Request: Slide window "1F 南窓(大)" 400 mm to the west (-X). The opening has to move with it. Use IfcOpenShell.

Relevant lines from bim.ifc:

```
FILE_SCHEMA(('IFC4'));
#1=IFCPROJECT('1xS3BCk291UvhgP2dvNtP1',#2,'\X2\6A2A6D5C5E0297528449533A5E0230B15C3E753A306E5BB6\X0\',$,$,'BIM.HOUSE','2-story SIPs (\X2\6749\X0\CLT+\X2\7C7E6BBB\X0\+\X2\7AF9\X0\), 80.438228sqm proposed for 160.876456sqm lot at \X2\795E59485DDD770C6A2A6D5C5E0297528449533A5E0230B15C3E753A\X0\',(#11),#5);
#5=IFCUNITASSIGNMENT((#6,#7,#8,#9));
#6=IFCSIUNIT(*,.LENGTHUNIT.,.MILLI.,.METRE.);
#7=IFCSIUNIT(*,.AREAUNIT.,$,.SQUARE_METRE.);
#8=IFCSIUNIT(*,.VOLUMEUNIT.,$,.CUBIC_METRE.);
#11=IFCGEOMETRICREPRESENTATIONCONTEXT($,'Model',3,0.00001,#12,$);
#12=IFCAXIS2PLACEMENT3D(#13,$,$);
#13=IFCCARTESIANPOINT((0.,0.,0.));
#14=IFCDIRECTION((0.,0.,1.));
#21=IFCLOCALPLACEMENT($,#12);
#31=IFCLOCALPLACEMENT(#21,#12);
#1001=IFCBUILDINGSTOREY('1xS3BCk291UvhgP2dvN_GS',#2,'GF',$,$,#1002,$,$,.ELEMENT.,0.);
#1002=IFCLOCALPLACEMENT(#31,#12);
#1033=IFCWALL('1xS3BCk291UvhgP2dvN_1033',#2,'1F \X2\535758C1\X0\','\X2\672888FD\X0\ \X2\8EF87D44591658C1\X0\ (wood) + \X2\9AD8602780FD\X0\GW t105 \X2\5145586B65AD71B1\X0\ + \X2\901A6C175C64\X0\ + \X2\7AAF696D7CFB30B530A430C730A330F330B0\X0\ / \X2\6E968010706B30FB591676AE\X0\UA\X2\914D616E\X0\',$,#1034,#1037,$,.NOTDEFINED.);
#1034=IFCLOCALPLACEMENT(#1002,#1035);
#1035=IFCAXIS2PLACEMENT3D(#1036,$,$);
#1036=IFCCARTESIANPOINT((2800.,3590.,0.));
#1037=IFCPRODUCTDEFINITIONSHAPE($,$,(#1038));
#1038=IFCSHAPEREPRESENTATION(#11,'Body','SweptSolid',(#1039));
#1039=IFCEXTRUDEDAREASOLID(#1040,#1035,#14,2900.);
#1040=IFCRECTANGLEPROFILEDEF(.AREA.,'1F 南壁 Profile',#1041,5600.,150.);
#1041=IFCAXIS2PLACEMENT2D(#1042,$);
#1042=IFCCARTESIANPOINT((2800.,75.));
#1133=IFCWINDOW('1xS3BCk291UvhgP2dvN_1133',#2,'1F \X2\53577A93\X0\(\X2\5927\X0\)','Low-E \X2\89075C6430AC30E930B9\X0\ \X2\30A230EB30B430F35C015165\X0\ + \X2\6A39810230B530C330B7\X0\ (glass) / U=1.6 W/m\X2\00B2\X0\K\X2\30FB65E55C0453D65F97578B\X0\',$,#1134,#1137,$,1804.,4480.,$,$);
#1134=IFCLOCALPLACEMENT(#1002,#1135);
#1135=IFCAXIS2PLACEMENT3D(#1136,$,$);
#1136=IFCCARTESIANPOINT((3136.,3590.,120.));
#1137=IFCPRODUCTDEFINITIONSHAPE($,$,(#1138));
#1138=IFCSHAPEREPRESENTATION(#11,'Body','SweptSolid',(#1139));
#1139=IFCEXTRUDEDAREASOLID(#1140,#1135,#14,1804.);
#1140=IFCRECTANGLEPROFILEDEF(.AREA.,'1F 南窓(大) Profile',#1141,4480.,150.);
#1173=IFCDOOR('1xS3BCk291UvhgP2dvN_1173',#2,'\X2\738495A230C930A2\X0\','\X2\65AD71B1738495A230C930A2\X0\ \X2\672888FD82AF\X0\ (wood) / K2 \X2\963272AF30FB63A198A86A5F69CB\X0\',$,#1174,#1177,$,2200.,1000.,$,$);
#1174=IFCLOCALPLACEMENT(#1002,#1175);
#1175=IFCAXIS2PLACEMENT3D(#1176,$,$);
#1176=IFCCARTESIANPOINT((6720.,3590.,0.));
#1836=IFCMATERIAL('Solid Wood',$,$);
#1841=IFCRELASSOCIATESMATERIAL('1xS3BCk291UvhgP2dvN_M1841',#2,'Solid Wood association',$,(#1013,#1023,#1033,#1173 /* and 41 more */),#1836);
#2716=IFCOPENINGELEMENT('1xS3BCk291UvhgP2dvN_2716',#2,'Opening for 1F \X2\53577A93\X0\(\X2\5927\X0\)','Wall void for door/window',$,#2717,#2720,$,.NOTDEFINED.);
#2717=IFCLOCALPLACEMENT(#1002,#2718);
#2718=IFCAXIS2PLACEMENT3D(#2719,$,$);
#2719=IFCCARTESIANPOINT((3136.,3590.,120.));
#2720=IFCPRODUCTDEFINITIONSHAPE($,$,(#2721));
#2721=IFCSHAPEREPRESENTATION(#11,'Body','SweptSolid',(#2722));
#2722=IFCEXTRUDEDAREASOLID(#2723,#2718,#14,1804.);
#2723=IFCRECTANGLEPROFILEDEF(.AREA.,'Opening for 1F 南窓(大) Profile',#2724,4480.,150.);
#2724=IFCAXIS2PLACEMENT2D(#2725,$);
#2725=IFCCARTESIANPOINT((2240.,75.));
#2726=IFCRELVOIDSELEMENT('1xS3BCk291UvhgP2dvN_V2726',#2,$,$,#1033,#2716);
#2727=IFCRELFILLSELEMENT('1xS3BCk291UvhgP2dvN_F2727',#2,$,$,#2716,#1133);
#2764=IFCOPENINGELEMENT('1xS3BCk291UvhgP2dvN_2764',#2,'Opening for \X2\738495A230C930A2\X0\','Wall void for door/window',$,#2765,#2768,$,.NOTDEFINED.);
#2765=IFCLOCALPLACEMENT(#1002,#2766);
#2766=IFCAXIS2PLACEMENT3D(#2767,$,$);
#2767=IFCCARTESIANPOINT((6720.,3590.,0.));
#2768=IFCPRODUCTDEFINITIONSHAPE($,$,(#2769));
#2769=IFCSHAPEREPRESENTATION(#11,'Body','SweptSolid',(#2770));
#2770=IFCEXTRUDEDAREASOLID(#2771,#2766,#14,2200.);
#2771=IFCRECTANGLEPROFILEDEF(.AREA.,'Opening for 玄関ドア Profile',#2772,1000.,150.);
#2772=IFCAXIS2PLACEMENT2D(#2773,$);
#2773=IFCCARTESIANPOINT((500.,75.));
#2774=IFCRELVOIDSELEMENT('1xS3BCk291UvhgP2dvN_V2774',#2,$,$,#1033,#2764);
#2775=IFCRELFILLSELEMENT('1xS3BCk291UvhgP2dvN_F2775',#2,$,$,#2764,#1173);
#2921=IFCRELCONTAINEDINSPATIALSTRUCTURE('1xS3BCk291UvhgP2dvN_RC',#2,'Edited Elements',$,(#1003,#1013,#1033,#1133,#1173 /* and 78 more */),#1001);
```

```python
import ifcopenshell
import ifcopenshell.api.geometry
import ifcopenshell.util.placement
import ifcopenshell.util.unit

model = ifcopenshell.open("bim.ifc")
unit_scale = ifcopenshell.util.unit.calculate_unit_scale(model)

window = model.by_id(1133)
opening = window.FillsVoids[0].RelatingOpeningElement
wall = opening.VoidsElements[0].RelatingBuildingElement

wall_matrix = ifcopenshell.util.placement.get_local_placement(wall.ObjectPlacement)
shift = wall_matrix[:3, 0] * -0.4 / unit_scale
before = ifcopenshell.util.placement.get_local_placement(window.ObjectPlacement)[:3, 3].copy()

# The window is not placed relative to its opening, so move both.
for product in (opening, window):
    matrix = ifcopenshell.util.placement.get_local_placement(product.ObjectPlacement)
    matrix[:3, 3] += shift
    ifcopenshell.api.geometry.edit_object_placement(model, product=product, matrix=matrix, is_si=False)

after = ifcopenshell.util.placement.get_local_placement(window.ObjectPlacement)[:3, 3]
print("window moved by", (after - before).round(3) + 0.0)

model.write("bim_rev.ifc")
```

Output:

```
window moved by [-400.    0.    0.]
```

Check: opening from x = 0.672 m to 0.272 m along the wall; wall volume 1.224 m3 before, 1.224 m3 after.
